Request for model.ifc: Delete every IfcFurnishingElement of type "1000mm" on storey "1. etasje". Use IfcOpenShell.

First a look at what the model holds.

```python
import ifcopenshell
import ifcopenshell.util.element

model = ifcopenshell.open("model.ifc")
print(model.schema)
storey = next(s for s in model.by_type("IfcBuildingStorey") if s.Name == "1. etasje")
furniture = [e for e in ifcopenshell.util.element.get_decomposition(storey) if e.is_a("IfcFurnishingElement")]
seen = {}
for e in furniture:
    element_type = ifcopenshell.util.element.get_type(e)
    name = element_type.Name if element_type not in (None, e) else None
    seen[name] = seen.get(name, 0) + 1
for name, count in sorted(seen.items(), key=str):
    print(count, "x", name)
```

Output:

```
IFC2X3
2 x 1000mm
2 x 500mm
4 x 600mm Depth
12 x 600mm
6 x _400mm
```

```python
import ifcopenshell
import ifcopenshell.api.root
import ifcopenshell.util.element

model = ifcopenshell.open("model.ifc")

storey = next(s for s in model.by_type("IfcBuildingStorey") if s.Name == "1. etasje")
furniture = [e for e in ifcopenshell.util.element.get_decomposition(storey) if e.is_a("IfcFurnishingElement")]
targets = [e for e in furniture if (t := ifcopenshell.util.element.get_type(e)) not in (None, e) and t.Name == "1000mm"]

for e in targets:
    ifcopenshell.api.root.remove_product(model, product=e)
print(len(targets), "removed")

model.write("model_v2.ifc")
```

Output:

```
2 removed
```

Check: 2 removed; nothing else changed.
